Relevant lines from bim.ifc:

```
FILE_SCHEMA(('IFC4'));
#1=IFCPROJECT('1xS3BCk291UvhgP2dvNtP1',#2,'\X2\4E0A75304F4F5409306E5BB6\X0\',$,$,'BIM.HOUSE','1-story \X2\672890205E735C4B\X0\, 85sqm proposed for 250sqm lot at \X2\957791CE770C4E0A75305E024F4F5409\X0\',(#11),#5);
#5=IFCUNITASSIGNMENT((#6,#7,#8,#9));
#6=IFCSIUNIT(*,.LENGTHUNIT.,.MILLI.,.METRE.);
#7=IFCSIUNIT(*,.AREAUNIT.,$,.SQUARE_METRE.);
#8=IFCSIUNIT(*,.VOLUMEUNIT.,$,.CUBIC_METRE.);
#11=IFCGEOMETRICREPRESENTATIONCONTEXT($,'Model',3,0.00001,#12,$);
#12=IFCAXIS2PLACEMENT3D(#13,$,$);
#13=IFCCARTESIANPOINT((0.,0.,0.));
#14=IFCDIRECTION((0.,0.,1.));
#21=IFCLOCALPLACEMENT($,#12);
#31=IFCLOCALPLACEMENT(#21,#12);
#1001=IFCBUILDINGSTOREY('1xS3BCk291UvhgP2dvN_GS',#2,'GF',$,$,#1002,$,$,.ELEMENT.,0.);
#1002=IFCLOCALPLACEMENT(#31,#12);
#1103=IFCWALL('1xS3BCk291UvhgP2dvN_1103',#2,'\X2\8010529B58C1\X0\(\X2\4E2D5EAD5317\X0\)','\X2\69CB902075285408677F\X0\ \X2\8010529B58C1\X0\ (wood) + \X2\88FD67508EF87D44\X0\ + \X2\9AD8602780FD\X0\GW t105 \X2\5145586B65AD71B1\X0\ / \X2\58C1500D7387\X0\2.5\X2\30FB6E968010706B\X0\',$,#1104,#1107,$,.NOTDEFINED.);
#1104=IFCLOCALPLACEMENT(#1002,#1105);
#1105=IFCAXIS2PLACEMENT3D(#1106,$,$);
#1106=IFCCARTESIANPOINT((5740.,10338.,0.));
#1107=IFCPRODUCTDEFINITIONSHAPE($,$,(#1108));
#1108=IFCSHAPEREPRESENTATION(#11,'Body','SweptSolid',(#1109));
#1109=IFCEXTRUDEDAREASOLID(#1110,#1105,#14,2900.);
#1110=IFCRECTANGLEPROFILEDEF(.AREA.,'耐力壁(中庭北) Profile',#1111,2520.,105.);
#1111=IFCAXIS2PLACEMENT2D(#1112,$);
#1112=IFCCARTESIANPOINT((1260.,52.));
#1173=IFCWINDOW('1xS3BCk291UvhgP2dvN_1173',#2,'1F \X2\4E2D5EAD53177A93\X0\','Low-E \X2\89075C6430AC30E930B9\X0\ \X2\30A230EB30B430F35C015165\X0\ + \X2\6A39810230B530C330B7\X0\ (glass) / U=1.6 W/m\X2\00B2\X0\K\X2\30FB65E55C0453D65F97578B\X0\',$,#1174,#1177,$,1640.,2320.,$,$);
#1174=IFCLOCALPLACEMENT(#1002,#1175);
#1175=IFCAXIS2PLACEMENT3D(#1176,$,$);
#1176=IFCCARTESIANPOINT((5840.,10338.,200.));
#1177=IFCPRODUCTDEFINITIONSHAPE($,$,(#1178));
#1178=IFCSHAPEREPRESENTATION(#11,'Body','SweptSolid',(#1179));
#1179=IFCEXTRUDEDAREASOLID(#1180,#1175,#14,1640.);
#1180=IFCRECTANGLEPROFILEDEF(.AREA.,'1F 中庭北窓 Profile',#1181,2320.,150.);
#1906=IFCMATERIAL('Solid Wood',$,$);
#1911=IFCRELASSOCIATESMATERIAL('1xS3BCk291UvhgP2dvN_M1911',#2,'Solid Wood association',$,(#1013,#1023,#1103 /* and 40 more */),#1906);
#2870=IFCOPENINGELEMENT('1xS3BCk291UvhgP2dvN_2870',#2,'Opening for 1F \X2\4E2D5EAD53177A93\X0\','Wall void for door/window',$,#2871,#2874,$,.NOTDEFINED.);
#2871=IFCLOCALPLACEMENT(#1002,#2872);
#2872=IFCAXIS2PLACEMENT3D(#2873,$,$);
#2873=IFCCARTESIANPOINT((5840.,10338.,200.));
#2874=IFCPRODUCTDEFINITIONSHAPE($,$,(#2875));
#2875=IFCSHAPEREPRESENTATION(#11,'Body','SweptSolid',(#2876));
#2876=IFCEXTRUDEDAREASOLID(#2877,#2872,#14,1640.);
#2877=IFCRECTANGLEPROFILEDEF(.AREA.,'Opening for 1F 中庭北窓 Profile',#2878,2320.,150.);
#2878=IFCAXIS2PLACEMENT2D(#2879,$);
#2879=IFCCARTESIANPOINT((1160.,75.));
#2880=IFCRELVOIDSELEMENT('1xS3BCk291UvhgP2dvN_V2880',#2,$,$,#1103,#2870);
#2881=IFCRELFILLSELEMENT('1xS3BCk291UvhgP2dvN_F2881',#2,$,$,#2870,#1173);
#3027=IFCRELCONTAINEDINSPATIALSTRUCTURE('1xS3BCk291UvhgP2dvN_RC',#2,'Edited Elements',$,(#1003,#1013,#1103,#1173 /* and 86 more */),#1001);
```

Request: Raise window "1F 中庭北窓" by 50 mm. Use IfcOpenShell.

```python
import numpy as np
import ifcopenshell
import ifcopenshell.api.geometry
import ifcopenshell.util.placement
import ifcopenshell.util.unit

model = ifcopenshell.open("bim.ifc")
unit_scale = ifcopenshell.util.unit.calculate_unit_scale(model)

window = model.by_guid("1xS3BCk291UvhgP2dvN_1173")
opening = window.FillsVoids[0].RelatingOpeningElement
dz = 0.05 / unit_scale

shift = np.array([0.0, 0.0, dz])
# The window is not placed relative to its opening, so move both.
for product in (opening, window):
    matrix = ifcopenshell.util.placement.get_local_placement(product.ObjectPlacement)
    matrix[:3, 3] += shift
    ifcopenshell.api.geometry.edit_object_placement(model, product=product, matrix=matrix, is_si=False)

print(f"moved by {dz * unit_scale:+.3f} m")

model.write("bim-out.ifc")
```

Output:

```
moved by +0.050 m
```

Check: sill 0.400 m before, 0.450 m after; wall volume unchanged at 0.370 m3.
